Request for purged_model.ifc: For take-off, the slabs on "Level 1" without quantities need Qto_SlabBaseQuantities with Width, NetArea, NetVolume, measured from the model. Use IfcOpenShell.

First a look at what the model holds.

```python
import ifcopenshell
import ifcopenshell.util.element
import ifcopenshell.util.unit

model = ifcopenshell.open("purged_model.ifc")
print(model.schema)
for unit_type in ("LENGTHUNIT", "AREAUNIT", "VOLUMEUNIT"):
    print(unit_type, ifcopenshell.util.unit.calculate_unit_scale(model, unit_type))
storey = next(s for s in model.by_type("IfcBuildingStorey") if s.Name == "Level 1")
slabs = [e for e in ifcopenshell.util.element.get_decomposition(storey) if e.is_a("IfcSlab")]
for e in sorted(slabs, key=lambda e: e.id()):
    print(e.id(), e.is_a(), e.Name, list(ifcopenshell.util.element.get_psets(e, qtos_only=True)), sep=" | ")
```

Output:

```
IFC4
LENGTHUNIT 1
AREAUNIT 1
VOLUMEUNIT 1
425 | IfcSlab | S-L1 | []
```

```python
import ifcopenshell
import ifcopenshell.api.pset
import ifcopenshell.geom
import ifcopenshell.util.element
import ifcopenshell.util.shape
import ifcopenshell.util.unit

model = ifcopenshell.open("purged_model.ifc")
unit_scale = ifcopenshell.util.unit.calculate_unit_scale(model)
area_scale = ifcopenshell.util.unit.calculate_unit_scale(model, "AREAUNIT")
volume_scale = ifcopenshell.util.unit.calculate_unit_scale(model, "VOLUMEUNIT")
settings = ifcopenshell.geom.settings()

storey = next(s for s in model.by_type("IfcBuildingStorey") if s.Name == "Level 1")
slabs = [e for e in ifcopenshell.util.element.get_decomposition(storey) if e.is_a("IfcSlab")]

for e in sorted(slabs, key=lambda e: e.id()):
    if ifcopenshell.util.element.get_psets(e, qtos_only=True, should_inherit=False):
        continue
    # Geometry comes back in metres, in the element's own axes.
    shape = ifcopenshell.geom.create_shape(settings, e)
    values = {
        "Width": ifcopenshell.util.shape.get_z(shape.geometry) / unit_scale,
        "NetArea": ifcopenshell.util.shape.get_footprint_area(shape.geometry) / area_scale,
        "NetVolume": ifcopenshell.util.shape.get_volume(shape.geometry) / volume_scale,
    }
    qto = ifcopenshell.api.pset.add_qto(model, product=e, name="Qto_SlabBaseQuantities")
    ifcopenshell.api.pset.edit_qto(model, qto=qto, properties=values)
    print(e.id(), {k: round(v, 3) for k, v in values.items()})

model.write("purged_model_updated.ifc")
```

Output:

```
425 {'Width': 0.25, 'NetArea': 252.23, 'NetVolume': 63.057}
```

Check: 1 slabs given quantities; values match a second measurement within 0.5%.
